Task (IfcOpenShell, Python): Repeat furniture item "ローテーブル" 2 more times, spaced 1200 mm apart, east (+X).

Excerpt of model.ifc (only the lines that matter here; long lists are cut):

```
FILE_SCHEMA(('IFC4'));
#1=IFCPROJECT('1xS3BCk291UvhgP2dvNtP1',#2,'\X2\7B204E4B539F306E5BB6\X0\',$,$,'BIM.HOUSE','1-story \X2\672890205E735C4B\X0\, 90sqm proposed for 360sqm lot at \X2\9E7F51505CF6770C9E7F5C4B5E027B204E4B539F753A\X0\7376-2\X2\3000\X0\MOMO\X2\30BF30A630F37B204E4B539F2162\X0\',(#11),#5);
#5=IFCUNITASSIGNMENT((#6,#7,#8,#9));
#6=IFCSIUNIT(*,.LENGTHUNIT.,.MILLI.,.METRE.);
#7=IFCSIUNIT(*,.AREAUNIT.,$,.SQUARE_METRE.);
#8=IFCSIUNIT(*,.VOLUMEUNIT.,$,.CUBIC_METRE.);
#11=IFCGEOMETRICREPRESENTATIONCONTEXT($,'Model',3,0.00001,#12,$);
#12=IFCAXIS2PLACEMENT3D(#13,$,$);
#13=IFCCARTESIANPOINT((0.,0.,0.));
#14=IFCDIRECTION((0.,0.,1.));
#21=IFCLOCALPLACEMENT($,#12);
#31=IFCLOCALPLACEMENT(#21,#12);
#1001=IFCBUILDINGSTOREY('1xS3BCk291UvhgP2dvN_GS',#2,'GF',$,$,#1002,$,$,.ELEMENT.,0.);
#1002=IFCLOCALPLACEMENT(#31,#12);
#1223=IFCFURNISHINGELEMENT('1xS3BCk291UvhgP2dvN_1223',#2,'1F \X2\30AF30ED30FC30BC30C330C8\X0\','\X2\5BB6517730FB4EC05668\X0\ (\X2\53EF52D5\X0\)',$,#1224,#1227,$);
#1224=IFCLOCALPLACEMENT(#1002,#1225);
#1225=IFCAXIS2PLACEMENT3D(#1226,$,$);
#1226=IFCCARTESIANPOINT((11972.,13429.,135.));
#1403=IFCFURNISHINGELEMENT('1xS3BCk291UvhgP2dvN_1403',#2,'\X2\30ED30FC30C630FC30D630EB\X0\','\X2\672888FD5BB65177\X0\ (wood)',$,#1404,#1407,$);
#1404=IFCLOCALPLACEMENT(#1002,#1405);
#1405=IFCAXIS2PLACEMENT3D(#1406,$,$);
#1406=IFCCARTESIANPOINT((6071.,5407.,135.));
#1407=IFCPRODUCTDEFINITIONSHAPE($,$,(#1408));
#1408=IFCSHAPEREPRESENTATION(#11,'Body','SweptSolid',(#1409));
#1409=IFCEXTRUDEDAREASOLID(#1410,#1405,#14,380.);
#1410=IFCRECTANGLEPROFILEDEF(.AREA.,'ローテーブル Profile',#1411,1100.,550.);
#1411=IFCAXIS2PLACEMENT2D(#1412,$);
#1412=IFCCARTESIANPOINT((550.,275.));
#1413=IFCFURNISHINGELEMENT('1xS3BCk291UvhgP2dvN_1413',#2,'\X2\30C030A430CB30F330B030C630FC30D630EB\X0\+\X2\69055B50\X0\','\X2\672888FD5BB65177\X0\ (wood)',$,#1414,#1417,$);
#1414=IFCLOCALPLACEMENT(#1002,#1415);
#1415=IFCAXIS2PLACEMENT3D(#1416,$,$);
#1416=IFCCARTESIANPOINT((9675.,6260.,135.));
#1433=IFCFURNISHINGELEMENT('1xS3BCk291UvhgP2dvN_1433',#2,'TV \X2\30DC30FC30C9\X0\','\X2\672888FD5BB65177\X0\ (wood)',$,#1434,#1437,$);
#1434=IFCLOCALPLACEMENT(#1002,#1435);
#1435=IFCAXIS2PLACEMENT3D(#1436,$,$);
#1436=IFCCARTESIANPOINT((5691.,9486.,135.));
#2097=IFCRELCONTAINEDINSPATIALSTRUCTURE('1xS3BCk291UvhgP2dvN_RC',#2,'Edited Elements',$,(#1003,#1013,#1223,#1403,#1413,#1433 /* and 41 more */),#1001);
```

```python
import numpy as np
import ifcopenshell
import ifcopenshell.api.geometry
import ifcopenshell.api.root
import ifcopenshell.util.element
import ifcopenshell.util.placement

model = ifcopenshell.open("model.ifc")


def reuse_history(source, copy):
    """copy_class also copies each property set's owner history, people and application; keep the originals."""
    for rel in copy.IsDefinedBy:
        if rel.is_a("IfcRelDefinesByProperties") and (history := rel.RelatingPropertyDefinition.OwnerHistory):
            rel.RelatingPropertyDefinition.OwnerHistory = source.OwnerHistory
            ifcopenshell.util.element.remove_deep2(model, history)


source = model.by_guid("1xS3BCk291UvhgP2dvN_1403")
base = ifcopenshell.util.placement.get_local_placement(source.ObjectPlacement)
step = np.array([1.0, 0.0, 0.0]) * 1200.0

for i in range(1, 3):
    copy = ifcopenshell.api.root.copy_class(model, product=source)
    copy.Representation = ifcopenshell.util.element.copy_deep(
        model, source.Representation, exclude=["IfcGeometricRepresentationContext", "IfcRepresentationMap"]
    )
    reuse_history(source, copy)
    matrix = base.copy()
    matrix[:3, 3] += i * step
    print("added at", matrix[:3, 3].round(3) + 0.0)
    ifcopenshell.api.geometry.edit_object_placement(model, product=copy, matrix=matrix, is_si=False)

model.write("model_v2.ifc")
```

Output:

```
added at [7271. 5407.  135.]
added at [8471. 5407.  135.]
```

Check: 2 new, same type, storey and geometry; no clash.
